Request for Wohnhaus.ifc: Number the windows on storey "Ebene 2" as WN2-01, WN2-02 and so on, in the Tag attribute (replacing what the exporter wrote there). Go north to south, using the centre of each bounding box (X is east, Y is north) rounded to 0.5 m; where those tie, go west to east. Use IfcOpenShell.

First a look at what the model holds.

```python
import ifcopenshell
import ifcopenshell.util.element
import ifcopenshell.util.placement

model = ifcopenshell.open("Wohnhaus.ifc")
print(model.schema)
storey = next(s for s in model.by_type("IfcBuildingStorey") if s.Name == "Ebene 2")
windows = [e for e in ifcopenshell.util.element.get_decomposition(storey) if e.is_a("IfcWindow")]
for e in sorted(windows, key=lambda e: e.id()):
    origin = ifcopenshell.util.placement.get_local_placement(e.ObjectPlacement)[:3, 3]
    print(e.id(), e.Tag, e.Name, origin.round(2) + 0.0, sep=" | ")
```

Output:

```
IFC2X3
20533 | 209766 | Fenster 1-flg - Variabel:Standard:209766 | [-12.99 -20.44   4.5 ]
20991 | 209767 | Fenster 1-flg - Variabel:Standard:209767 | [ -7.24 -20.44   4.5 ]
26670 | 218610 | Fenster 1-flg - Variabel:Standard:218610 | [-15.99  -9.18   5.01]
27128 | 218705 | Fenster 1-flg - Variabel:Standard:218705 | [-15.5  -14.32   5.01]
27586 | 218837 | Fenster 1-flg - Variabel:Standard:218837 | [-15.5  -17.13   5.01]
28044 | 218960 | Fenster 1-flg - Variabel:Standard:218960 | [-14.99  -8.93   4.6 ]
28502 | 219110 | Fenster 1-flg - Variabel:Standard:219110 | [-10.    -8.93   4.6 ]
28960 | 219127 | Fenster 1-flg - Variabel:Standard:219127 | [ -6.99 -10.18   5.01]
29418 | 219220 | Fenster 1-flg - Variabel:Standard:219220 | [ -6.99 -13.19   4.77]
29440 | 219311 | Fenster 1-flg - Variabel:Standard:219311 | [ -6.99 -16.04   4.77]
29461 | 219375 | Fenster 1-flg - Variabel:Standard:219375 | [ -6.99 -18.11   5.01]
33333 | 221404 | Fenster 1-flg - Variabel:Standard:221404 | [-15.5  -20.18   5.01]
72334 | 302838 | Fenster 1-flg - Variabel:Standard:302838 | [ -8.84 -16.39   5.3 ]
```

```python
import ifcopenshell
import ifcopenshell.geom
import ifcopenshell.util.element
import ifcopenshell.util.shape

model = ifcopenshell.open("Wohnhaus.ifc")
settings = ifcopenshell.geom.settings()
settings.set("use-world-coords", True)


def centre(element):
    shape = ifcopenshell.geom.create_shape(settings, element)
    return ifcopenshell.util.shape.get_bbox_centroid(shape.geometry)


storey = next(s for s in model.by_type("IfcBuildingStorey") if s.Name == "Ebene 2")
windows = [e for e in ifcopenshell.util.element.get_decomposition(storey) if e.is_a("IfcWindow")]

# Insertion points can sit at a corner or the storey origin, so sort by the geometry (in metres).
centres = {e: centre(e) for e in windows}
windows.sort(key=lambda e: (-round(centres[e][1] / 0.5), centres[e][0]))

for i, e in enumerate(windows, start=1):
    number = f"WN2-{i:02d}"
    e.Tag = number
    print(e.id(), number)

model.write("Wohnhaus_v2.ifc")
```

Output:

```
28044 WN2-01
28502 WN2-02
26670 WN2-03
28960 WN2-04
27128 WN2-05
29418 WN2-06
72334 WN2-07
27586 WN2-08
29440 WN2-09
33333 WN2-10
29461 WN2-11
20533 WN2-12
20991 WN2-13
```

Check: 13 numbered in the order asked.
